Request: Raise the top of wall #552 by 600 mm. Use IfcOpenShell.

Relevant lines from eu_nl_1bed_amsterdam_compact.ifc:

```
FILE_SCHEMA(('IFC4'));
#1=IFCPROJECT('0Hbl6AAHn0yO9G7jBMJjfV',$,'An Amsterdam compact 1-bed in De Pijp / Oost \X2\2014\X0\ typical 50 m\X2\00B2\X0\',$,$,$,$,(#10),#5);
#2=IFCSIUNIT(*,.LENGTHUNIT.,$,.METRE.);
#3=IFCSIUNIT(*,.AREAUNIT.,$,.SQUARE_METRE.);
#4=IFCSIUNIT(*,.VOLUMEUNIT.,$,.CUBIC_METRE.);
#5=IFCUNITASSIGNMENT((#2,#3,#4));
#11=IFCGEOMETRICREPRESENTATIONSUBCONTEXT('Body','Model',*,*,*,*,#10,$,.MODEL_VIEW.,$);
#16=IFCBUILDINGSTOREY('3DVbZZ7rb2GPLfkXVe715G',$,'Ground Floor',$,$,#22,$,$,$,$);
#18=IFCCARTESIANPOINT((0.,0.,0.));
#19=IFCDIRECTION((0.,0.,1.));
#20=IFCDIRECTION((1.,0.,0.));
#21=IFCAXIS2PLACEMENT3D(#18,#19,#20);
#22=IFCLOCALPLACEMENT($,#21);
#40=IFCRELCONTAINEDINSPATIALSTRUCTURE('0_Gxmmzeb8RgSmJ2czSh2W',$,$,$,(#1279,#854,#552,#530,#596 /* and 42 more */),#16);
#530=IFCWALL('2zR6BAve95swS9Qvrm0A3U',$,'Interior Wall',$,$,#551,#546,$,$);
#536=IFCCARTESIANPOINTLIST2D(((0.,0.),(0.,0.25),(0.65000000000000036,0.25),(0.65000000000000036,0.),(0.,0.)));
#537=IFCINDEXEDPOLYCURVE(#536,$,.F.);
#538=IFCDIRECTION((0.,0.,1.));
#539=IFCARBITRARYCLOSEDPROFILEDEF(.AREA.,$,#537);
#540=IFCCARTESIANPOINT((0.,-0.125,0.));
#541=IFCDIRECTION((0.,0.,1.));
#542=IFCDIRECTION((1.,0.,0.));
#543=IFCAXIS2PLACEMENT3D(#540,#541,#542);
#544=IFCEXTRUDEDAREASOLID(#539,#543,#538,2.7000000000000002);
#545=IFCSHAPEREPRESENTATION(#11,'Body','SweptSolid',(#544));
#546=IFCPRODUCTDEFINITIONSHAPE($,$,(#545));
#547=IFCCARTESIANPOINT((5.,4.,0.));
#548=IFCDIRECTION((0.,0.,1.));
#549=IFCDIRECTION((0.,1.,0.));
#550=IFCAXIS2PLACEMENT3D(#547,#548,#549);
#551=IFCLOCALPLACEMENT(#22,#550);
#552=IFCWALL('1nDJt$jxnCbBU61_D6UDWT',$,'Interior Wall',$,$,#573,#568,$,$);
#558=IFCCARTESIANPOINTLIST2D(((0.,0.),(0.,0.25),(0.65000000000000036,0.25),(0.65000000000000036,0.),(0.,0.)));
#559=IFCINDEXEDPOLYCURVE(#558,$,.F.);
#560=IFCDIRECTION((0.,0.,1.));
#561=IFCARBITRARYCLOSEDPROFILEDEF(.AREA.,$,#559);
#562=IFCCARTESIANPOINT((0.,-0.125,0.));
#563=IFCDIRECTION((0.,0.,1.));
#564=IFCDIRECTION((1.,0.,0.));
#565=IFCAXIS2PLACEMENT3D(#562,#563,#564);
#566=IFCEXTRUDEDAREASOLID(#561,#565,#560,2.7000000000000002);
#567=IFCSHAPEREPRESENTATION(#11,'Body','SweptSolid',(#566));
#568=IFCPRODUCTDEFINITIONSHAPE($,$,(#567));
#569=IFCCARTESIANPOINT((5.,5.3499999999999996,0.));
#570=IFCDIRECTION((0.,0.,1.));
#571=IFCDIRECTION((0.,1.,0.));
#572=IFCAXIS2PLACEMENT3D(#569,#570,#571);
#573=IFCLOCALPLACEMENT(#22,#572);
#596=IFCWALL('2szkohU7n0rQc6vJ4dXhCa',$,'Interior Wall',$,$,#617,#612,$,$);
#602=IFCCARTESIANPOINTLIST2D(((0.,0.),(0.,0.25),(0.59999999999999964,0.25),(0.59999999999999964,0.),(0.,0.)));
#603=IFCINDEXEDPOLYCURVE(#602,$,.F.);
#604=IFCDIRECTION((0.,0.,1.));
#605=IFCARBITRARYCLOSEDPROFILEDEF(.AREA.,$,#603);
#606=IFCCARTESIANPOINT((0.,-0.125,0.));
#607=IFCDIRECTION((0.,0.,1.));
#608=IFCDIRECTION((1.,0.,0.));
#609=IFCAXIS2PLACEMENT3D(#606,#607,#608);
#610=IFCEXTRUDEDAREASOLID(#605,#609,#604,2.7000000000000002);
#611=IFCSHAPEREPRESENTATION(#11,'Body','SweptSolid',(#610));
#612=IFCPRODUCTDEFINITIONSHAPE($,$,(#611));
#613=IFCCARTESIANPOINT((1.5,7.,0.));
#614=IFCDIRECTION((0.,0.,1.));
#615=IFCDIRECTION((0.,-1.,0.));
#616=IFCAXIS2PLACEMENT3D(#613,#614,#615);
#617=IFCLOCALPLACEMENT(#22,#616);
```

```python
import ifcopenshell
import ifcopenshell.geom
import ifcopenshell.util.representation
import ifcopenshell.util.shape
import ifcopenshell.util.unit

model = ifcopenshell.open("eu_nl_1bed_amsterdam_compact.ifc")
unit_scale = ifcopenshell.util.unit.calculate_unit_scale(model)
settings = ifcopenshell.geom.settings()


def volume(element):
    """Net volume in cubic metres, openings subtracted."""
    shape = ifcopenshell.geom.create_shape(settings, element)
    return ifcopenshell.util.shape.get_volume(shape.geometry)


wall = model.by_guid("1nDJt$jxnCbBU61_D6UDWT")
before = volume(wall)

body = ifcopenshell.util.representation.get_representation(wall, "Model", "Body")
solid = body.Items[0]
old_height = solid.Depth
solid.Depth += 0.6 / unit_scale
after = volume(wall)

print(f"height {old_height:g} -> {solid.Depth:g}, volume {before:.3f} -> {after:.3f} m3")

model.write("eu_nl_1bed_amsterdam_compact_v2.ifc")
```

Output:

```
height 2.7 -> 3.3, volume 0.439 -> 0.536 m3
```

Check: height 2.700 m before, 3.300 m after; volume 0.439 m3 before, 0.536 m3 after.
